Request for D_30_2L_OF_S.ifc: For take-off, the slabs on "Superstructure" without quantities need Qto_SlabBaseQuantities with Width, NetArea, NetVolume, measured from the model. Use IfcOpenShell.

First a look at what the model holds.

```python
import ifcopenshell
import ifcopenshell.util.element
import ifcopenshell.util.unit

model = ifcopenshell.open("D_30_2L_OF_S.ifc")
print(model.schema)
for unit_type in ("LENGTHUNIT", "AREAUNIT", "VOLUMEUNIT"):
    print(unit_type, ifcopenshell.util.unit.calculate_unit_scale(model, unit_type))
storey = next(s for s in model.by_type("IfcBuildingStorey") if s.Name == "Superstructure")
slabs = [e for e in ifcopenshell.util.element.get_decomposition(storey) if e.is_a("IfcSlab")]
for e in sorted(slabs, key=lambda e: e.id()):
    print(e.id(), e.is_a(), e.Name, list(ifcopenshell.util.element.get_psets(e, qtos_only=True)), sep=" | ")
```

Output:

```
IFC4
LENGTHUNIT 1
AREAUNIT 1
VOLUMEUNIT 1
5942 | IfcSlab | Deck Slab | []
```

```python
import ifcopenshell
import ifcopenshell.api.pset
import ifcopenshell.geom
import ifcopenshell.util.element
import ifcopenshell.util.shape
import ifcopenshell.util.unit

model = ifcopenshell.open("D_30_2L_OF_S.ifc")
unit_scale = ifcopenshell.util.unit.calculate_unit_scale(model)
area_scale = ifcopenshell.util.unit.calculate_unit_scale(model, "AREAUNIT")
volume_scale = ifcopenshell.util.unit.calculate_unit_scale(model, "VOLUMEUNIT")
settings = ifcopenshell.geom.settings()

storey = next(s for s in model.by_type("IfcBuildingStorey") if s.Name == "Superstructure")
slabs = [e for e in ifcopenshell.util.element.get_decomposition(storey) if e.is_a("IfcSlab")]

for e in sorted(slabs, key=lambda e: e.id()):
    if ifcopenshell.util.element.get_psets(e, qtos_only=True, should_inherit=False):
        continue
    # Geometry comes back in metres, in the element's own axes.
    shape = ifcopenshell.geom.create_shape(settings, e)
    values = {
        "Width": ifcopenshell.util.shape.get_z(shape.geometry) / unit_scale,
        "NetArea": ifcopenshell.util.shape.get_footprint_area(shape.geometry) / area_scale,
        "NetVolume": ifcopenshell.util.shape.get_volume(shape.geometry) / volume_scale,
    }
    qto = ifcopenshell.api.pset.add_qto(model, product=e, name="Qto_SlabBaseQuantities")
    ifcopenshell.api.pset.edit_qto(model, qto=qto, properties=values)
    print(e.id(), {k: round(v, 3) for k, v in values.items()})

model.write("D_30_2L_OF_S_v2.ifc")
```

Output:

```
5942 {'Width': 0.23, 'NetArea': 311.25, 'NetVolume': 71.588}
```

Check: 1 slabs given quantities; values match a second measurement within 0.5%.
